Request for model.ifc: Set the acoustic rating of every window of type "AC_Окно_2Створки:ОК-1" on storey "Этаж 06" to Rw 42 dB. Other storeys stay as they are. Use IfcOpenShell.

First a look at what the model holds.

```python
import ifcopenshell
import ifcopenshell.util.element

model = ifcopenshell.open("model.ifc")
print(model.schema)
storey = next(s for s in model.by_type("IfcBuildingStorey") if s.Name == "Этаж 06")
windows = [e for e in ifcopenshell.util.element.get_decomposition(storey) if e.is_a("IfcWindow")]
seen = {}
for e in windows:
    element_type = ifcopenshell.util.element.get_type(e)
    key = (element_type.Name if element_type != e and element_type else None, ifcopenshell.util.element.get_pset(e, "Pset_WindowCommon", "AcousticRating"))
    seen[key] = seen.get(key, 0) + 1
for (name, value), count in sorted(seen.items(), key=str):
    print(count, "x", name, "|", value)
```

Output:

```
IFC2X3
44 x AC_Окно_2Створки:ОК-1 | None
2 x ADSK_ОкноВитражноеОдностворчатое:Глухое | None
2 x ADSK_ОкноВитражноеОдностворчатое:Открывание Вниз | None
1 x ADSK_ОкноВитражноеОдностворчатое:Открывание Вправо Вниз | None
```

```python
import ifcopenshell
import ifcopenshell.api.pset
import ifcopenshell.util.element

model = ifcopenshell.open("model.ifc")

storey = next(s for s in model.by_type("IfcBuildingStorey") if s.Name == "Этаж 06")
windows = [e for e in ifcopenshell.util.element.get_decomposition(storey) if e.is_a("IfcWindow")]

count = 0
for e in windows:
    element_type = ifcopenshell.util.element.get_type(e)
    if element_type in (None, e) or element_type.Name != "AC_Окно_2Створки:ОК-1":
        continue
    # add_pset returns the element's existing set when there is one.
    pset = ifcopenshell.api.pset.add_pset(model, product=e, name="Pset_WindowCommon")
    ifcopenshell.api.pset.edit_pset(model, pset=pset, properties={"AcousticRating": "Rw 42 dB"})
    count += 1

print(count, "windows updated")

model.write("model_rev.ifc")
```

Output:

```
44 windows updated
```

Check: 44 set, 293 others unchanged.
